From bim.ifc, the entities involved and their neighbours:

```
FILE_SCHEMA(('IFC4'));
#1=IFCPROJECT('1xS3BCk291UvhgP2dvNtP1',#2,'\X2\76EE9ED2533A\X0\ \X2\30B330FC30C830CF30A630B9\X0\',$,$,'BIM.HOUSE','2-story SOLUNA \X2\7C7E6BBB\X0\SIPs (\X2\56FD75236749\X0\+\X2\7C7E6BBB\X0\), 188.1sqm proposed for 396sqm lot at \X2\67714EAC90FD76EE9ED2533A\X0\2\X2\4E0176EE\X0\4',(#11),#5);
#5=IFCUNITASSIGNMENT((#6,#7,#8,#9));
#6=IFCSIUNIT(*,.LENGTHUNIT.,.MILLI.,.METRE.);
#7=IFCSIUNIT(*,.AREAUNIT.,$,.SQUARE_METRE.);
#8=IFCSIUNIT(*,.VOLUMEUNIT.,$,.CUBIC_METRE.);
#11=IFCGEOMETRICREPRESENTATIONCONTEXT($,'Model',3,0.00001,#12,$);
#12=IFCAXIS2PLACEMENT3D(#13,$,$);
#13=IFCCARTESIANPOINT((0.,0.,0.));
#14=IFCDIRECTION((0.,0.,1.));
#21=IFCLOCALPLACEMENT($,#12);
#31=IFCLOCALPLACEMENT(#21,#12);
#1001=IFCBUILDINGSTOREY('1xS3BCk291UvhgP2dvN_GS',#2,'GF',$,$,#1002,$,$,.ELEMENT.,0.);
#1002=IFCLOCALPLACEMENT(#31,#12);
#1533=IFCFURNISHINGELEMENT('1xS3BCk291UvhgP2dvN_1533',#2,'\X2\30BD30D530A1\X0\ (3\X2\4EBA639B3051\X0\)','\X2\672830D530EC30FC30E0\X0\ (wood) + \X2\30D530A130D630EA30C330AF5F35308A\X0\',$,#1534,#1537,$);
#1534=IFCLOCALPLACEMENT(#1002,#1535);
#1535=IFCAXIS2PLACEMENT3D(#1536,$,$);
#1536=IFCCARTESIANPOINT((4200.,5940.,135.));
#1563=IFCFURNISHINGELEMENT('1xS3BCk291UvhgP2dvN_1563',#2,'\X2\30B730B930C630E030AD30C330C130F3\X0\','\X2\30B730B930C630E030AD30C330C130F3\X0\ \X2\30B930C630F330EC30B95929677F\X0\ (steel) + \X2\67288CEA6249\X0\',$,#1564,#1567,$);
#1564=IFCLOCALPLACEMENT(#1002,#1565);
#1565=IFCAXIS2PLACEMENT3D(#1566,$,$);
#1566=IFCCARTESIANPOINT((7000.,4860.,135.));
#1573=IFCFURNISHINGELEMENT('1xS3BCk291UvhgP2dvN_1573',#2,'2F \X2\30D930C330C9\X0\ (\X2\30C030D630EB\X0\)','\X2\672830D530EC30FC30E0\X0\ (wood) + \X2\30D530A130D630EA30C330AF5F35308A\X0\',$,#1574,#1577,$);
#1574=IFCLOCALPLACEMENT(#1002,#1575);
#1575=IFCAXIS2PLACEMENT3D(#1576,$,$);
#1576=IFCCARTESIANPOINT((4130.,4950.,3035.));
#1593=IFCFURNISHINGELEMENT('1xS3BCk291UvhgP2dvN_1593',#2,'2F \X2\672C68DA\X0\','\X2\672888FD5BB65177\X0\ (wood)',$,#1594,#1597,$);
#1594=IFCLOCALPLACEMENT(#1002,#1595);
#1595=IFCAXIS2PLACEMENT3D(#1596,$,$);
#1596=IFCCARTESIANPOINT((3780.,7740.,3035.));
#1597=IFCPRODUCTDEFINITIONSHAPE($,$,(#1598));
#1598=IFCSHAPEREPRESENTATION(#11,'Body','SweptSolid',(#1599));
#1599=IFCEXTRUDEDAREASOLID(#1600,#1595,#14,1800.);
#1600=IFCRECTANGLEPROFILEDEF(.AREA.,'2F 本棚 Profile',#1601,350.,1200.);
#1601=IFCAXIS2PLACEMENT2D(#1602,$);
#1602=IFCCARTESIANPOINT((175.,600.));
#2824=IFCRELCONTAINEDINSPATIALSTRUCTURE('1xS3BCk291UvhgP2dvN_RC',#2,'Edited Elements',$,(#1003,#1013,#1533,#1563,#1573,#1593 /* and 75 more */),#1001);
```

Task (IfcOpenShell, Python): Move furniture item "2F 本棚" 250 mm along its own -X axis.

```python
import ifcopenshell
import ifcopenshell.api.geometry
import ifcopenshell.util.placement
import ifcopenshell.util.unit

model = ifcopenshell.open("bim.ifc")
unit_scale = ifcopenshell.util.unit.calculate_unit_scale(model)

item = model.by_guid("1xS3BCk291UvhgP2dvN_1593")
matrix = ifcopenshell.util.placement.get_local_placement(item.ObjectPlacement)
matrix[:3, 3] -= matrix[:3, 0] * 0.25 / unit_scale
ifcopenshell.api.geometry.edit_object_placement(model, product=item, matrix=matrix, is_si=False)

print(ifcopenshell.util.placement.get_local_placement(item.ObjectPlacement).round(3) + 0.0)

model.write("bim-out.ifc")
```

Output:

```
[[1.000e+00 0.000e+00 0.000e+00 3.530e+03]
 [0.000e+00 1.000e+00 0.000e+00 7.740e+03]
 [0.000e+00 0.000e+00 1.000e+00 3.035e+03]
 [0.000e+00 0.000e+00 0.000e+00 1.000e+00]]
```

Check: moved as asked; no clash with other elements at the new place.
